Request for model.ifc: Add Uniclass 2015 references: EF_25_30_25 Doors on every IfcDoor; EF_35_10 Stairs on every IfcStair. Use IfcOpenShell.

First a look at what the model holds.

```python
import ifcopenshell

model = ifcopenshell.open("model.ifc")
print(model.schema)
print("classifications:", [c.Name for c in model.by_type("IfcClassification")])
for ifc_class in ("IfcDoor", "IfcRoof", "IfcStair", "IfcWall", "IfcWindow"):
    print(ifc_class, len(model.by_type(ifc_class)))
```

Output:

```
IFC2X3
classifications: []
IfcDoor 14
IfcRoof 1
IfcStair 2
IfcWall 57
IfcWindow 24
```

```python
import ifcopenshell
import ifcopenshell.api.classification

model = ifcopenshell.open("model.ifc")

# IFC2X3 requires Source and Edition and has no link from the project to the system.
system = model.create_entity("IfcClassification", Source="NBS", Edition="2015", Name="Uniclass 2015")

codes = {
    "IfcDoor": ("EF_25_30_25", "Doors"),
    "IfcStair": ("EF_35_10", "Stairs"),
}
for ifc_class, (code, name) in codes.items():
    products = model.by_type(ifc_class)
    ifcopenshell.api.classification.add_reference(
        model, products=products, classification=system, identification=code, name=name
    )
    print(code, len(products))

model.write("model_v2.ifc")
```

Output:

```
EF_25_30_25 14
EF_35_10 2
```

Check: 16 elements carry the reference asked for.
